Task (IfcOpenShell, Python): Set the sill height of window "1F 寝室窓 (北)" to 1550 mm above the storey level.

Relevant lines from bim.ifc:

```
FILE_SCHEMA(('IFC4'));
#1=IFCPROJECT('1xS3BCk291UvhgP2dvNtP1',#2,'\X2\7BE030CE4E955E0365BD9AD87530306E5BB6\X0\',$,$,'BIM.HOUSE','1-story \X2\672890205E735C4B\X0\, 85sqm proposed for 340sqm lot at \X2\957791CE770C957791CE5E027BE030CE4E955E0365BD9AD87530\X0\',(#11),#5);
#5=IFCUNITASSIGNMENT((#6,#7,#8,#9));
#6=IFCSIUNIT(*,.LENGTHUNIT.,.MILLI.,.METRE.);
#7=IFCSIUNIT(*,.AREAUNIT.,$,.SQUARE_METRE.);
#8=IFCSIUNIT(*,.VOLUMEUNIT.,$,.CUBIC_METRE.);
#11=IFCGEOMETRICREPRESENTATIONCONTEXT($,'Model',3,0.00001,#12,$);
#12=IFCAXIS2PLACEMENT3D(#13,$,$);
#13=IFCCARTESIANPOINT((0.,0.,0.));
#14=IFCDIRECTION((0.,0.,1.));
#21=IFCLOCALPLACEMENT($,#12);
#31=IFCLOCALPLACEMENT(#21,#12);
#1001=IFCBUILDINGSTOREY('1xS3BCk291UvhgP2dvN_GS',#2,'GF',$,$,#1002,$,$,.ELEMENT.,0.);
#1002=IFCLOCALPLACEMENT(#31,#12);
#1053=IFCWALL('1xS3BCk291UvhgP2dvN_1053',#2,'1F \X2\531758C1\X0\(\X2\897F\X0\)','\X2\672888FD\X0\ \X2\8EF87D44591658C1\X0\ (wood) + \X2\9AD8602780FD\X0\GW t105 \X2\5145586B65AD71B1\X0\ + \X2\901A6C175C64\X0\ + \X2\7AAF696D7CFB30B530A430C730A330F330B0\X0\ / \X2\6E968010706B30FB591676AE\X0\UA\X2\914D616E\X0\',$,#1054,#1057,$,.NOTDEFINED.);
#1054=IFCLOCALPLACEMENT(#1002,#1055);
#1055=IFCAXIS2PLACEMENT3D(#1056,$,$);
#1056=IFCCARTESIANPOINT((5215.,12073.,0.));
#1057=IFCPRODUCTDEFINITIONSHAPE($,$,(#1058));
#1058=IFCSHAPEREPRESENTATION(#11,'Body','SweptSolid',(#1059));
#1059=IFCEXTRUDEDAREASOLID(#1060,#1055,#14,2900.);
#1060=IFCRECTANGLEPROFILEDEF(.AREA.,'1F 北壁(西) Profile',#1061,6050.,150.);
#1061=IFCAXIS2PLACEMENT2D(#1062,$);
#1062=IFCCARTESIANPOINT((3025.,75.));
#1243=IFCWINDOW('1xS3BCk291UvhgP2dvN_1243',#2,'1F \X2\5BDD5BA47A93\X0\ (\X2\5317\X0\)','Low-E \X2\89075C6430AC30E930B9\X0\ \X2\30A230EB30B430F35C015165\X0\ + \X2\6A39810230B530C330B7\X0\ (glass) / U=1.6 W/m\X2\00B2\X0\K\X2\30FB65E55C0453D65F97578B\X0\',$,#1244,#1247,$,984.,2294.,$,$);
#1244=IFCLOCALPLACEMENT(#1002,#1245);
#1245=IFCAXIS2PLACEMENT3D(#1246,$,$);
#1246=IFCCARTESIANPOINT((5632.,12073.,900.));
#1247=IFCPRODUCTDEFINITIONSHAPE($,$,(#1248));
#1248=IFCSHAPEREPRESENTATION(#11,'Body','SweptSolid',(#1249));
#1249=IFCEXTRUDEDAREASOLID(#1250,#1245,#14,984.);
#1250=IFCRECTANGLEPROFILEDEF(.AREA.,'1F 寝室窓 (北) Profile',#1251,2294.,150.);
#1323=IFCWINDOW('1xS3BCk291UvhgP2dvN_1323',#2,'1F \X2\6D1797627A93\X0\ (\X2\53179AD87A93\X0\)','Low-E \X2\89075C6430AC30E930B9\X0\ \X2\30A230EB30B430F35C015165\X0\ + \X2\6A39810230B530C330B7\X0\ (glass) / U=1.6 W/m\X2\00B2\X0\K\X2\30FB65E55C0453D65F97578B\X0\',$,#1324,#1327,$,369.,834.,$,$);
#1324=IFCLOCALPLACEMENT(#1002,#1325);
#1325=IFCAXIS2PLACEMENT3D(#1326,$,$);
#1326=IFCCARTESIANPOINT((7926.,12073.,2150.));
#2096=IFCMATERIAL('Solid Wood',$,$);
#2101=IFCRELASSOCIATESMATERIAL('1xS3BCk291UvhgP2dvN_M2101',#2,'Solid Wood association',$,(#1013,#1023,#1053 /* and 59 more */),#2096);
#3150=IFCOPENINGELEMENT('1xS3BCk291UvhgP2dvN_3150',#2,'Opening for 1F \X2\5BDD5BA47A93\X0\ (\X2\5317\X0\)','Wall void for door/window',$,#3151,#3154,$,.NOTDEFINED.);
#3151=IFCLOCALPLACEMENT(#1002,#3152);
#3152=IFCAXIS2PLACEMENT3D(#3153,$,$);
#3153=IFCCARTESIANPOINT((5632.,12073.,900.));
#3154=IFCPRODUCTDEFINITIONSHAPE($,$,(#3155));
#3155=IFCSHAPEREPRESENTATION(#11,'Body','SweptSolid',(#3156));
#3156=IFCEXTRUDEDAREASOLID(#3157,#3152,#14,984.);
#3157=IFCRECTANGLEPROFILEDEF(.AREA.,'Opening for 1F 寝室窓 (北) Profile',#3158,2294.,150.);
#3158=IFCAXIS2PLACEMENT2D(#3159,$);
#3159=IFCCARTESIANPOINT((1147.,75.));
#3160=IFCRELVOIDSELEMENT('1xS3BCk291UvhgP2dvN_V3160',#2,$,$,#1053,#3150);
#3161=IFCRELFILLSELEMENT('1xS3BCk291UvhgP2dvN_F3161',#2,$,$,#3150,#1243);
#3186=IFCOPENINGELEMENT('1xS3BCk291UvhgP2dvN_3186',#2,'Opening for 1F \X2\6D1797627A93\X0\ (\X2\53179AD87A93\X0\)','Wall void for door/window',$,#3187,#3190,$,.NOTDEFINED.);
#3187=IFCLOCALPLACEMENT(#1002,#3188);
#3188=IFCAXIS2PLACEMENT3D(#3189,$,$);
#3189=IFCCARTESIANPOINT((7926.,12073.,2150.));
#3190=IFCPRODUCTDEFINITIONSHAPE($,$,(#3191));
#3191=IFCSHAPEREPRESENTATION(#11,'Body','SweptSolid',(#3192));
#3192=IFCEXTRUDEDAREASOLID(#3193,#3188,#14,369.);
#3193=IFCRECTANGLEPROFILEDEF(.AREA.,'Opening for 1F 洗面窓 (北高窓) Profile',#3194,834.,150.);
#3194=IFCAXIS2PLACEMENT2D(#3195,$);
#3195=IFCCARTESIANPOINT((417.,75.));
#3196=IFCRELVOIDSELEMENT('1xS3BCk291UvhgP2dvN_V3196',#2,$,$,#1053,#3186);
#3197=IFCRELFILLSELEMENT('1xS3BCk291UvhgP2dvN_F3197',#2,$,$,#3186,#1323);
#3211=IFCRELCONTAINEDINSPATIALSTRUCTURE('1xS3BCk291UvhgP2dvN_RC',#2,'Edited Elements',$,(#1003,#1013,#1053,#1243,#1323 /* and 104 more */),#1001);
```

```python
import numpy as np
import ifcopenshell
import ifcopenshell.api.geometry
import ifcopenshell.geom
import ifcopenshell.util.element
import ifcopenshell.util.placement
import ifcopenshell.util.shape
import ifcopenshell.util.unit

model = ifcopenshell.open("bim.ifc")
unit_scale = ifcopenshell.util.unit.calculate_unit_scale(model)

window = model.by_id(1243)
opening = window.FillsVoids[0].RelatingOpeningElement
storey = ifcopenshell.util.element.get_container(window, ifc_class="IfcBuildingStorey")
level = ifcopenshell.util.placement.get_local_placement(storey.ObjectPlacement)[2, 3]

# The opening's origin need not be at the sill, so measure its lowest point.
shape = ifcopenshell.geom.create_shape(ifcopenshell.geom.settings(), opening)
bottom = ifcopenshell.util.shape.get_shape_bottom_elevation(shape, shape.geometry) / unit_scale
dz = level + 1.55 / unit_scale - bottom

shift = np.array([0.0, 0.0, dz])
# The window is not placed relative to its opening, so move both.
for product in (opening, window):
    matrix = ifcopenshell.util.placement.get_local_placement(product.ObjectPlacement)
    matrix[:3, 3] += shift
    ifcopenshell.api.geometry.edit_object_placement(model, product=product, matrix=matrix, is_si=False)

print(f"moved by {dz * unit_scale:+.3f} m")

model.write("bim_rev.ifc")
```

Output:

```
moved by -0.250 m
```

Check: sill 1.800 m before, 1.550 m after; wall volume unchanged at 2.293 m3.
